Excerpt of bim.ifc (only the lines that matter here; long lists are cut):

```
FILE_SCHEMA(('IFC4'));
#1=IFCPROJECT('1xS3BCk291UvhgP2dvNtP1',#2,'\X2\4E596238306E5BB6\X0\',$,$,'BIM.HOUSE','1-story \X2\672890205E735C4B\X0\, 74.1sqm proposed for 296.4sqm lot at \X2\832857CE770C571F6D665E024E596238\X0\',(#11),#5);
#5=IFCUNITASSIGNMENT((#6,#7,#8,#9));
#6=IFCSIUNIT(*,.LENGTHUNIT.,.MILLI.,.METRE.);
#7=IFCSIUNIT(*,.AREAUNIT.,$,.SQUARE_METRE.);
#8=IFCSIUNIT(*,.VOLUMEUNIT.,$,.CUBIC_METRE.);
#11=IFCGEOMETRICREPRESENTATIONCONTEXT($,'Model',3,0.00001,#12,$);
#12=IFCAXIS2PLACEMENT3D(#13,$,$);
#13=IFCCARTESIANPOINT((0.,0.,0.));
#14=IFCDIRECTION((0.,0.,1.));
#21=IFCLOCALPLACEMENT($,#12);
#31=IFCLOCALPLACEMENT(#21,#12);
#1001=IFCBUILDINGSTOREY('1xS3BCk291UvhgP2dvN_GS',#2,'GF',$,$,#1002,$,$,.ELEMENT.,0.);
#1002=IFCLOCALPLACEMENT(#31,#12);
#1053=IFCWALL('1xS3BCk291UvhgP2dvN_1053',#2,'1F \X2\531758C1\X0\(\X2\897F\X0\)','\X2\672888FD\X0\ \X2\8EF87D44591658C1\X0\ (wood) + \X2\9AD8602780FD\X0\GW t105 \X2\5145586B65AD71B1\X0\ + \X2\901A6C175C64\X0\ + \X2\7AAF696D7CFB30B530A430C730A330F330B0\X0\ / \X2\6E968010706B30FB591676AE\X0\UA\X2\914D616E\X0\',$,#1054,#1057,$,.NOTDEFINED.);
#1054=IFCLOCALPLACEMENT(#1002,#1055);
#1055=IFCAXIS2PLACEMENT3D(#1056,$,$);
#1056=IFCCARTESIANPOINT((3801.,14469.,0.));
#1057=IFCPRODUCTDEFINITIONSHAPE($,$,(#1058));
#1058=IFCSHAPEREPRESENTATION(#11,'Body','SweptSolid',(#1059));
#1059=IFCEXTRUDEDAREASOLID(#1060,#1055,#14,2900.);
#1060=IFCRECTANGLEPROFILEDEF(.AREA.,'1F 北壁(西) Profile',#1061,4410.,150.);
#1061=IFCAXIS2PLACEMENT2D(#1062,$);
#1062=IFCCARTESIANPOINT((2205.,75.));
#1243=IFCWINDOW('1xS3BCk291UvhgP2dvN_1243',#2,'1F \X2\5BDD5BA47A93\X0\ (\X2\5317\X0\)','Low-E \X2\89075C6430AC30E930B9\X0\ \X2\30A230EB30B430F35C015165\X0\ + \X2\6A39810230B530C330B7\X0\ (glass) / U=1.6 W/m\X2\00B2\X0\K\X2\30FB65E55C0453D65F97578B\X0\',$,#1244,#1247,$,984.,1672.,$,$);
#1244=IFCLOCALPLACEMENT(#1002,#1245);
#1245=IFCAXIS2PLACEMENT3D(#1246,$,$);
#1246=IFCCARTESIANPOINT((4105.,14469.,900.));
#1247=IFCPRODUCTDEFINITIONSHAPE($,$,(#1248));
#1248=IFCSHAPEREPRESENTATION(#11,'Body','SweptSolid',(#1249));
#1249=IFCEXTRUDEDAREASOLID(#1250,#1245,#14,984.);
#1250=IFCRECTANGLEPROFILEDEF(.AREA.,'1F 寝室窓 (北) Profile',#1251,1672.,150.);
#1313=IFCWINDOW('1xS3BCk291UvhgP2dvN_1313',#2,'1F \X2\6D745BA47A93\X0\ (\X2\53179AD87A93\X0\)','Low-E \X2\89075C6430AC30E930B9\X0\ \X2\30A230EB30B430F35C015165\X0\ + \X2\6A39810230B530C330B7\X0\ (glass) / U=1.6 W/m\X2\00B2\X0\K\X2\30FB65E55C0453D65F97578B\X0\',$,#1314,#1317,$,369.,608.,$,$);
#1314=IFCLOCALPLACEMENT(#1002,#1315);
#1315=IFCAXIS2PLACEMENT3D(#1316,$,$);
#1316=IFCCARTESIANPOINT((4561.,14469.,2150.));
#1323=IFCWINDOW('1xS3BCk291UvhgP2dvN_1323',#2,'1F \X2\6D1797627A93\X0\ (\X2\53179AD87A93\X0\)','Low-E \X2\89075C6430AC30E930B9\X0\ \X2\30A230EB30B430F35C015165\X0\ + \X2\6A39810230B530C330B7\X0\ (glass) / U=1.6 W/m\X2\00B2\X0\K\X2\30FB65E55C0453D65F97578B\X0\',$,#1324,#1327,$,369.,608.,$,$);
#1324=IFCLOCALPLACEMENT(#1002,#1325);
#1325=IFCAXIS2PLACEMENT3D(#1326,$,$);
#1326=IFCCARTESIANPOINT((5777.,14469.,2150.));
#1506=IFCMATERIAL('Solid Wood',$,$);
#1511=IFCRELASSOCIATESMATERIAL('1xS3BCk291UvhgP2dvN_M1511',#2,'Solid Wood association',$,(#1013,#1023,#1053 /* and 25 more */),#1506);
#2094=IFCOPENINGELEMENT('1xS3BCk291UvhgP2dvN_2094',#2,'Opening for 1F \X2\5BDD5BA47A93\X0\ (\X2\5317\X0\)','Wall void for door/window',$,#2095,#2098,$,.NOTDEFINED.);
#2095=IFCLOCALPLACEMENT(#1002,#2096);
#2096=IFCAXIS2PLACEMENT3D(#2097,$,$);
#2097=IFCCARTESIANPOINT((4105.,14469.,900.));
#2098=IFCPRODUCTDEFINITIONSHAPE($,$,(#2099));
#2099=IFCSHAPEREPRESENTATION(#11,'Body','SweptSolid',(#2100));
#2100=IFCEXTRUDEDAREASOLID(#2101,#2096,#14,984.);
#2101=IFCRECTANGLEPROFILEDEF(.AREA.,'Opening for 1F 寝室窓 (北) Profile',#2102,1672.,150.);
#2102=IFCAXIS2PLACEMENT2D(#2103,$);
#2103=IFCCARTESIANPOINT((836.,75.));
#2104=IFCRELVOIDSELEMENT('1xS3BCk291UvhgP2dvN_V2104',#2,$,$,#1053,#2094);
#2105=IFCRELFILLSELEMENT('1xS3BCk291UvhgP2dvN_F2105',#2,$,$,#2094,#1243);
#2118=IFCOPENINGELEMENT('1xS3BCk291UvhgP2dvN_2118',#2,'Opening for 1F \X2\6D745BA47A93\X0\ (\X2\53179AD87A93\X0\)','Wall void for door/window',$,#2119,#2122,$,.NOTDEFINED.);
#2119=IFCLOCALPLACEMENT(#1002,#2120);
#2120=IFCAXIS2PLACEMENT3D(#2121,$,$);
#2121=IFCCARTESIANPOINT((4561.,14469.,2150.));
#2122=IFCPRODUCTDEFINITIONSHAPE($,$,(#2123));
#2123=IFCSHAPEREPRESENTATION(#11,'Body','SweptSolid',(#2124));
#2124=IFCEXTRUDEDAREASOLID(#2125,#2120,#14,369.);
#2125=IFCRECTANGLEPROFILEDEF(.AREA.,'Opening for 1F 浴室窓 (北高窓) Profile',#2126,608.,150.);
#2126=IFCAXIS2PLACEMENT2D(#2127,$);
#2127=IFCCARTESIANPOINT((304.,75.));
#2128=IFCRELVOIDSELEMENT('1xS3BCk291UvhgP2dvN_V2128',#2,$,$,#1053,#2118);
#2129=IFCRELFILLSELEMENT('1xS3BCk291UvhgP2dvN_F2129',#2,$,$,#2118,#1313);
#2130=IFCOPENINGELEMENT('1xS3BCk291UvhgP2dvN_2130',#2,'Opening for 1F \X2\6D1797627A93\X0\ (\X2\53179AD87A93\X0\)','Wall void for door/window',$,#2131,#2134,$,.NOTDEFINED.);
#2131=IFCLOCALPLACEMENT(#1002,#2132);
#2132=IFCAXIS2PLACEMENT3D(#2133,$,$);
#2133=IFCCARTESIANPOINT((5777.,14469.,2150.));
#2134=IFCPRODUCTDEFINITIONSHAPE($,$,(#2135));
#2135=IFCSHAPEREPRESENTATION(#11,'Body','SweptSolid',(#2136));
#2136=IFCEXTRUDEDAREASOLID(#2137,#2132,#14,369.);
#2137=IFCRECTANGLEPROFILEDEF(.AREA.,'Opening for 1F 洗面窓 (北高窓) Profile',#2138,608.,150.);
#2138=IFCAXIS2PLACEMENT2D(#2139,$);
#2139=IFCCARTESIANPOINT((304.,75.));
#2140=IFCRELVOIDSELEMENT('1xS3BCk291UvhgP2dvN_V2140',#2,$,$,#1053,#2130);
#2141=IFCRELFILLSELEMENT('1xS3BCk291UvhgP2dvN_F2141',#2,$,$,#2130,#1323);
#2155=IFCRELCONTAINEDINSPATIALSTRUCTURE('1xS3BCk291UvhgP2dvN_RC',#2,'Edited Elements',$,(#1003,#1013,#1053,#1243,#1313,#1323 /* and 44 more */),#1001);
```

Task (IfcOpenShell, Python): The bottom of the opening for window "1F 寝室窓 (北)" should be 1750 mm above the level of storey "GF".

```python
import numpy as np
import ifcopenshell
import ifcopenshell.api.geometry
import ifcopenshell.geom
import ifcopenshell.util.element
import ifcopenshell.util.placement
import ifcopenshell.util.shape
import ifcopenshell.util.unit

model = ifcopenshell.open("bim.ifc")
unit_scale = ifcopenshell.util.unit.calculate_unit_scale(model)

window = model.by_guid("1xS3BCk291UvhgP2dvN_1243")
opening = window.FillsVoids[0].RelatingOpeningElement
storey = ifcopenshell.util.element.get_container(window, ifc_class="IfcBuildingStorey")
level = ifcopenshell.util.placement.get_local_placement(storey.ObjectPlacement)[2, 3]

# The opening's origin need not be at the sill, so measure its lowest point.
shape = ifcopenshell.geom.create_shape(ifcopenshell.geom.settings(), opening)
bottom = ifcopenshell.util.shape.get_shape_bottom_elevation(shape, shape.geometry) / unit_scale
dz = level + 1750.0 - bottom

shift = np.array([0.0, 0.0, dz])
# The window is not placed relative to its opening, so move both.
for product in (opening, window):
    matrix = ifcopenshell.util.placement.get_local_placement(product.ObjectPlacement)
    matrix[:3, 3] += shift
    ifcopenshell.api.geometry.edit_object_placement(model, product=product, matrix=matrix, is_si=False)

print(f"moved by {dz * unit_scale:+.3f} m")

model.write("bim_v2.ifc")
```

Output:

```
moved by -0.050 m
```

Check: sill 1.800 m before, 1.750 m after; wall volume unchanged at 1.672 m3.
